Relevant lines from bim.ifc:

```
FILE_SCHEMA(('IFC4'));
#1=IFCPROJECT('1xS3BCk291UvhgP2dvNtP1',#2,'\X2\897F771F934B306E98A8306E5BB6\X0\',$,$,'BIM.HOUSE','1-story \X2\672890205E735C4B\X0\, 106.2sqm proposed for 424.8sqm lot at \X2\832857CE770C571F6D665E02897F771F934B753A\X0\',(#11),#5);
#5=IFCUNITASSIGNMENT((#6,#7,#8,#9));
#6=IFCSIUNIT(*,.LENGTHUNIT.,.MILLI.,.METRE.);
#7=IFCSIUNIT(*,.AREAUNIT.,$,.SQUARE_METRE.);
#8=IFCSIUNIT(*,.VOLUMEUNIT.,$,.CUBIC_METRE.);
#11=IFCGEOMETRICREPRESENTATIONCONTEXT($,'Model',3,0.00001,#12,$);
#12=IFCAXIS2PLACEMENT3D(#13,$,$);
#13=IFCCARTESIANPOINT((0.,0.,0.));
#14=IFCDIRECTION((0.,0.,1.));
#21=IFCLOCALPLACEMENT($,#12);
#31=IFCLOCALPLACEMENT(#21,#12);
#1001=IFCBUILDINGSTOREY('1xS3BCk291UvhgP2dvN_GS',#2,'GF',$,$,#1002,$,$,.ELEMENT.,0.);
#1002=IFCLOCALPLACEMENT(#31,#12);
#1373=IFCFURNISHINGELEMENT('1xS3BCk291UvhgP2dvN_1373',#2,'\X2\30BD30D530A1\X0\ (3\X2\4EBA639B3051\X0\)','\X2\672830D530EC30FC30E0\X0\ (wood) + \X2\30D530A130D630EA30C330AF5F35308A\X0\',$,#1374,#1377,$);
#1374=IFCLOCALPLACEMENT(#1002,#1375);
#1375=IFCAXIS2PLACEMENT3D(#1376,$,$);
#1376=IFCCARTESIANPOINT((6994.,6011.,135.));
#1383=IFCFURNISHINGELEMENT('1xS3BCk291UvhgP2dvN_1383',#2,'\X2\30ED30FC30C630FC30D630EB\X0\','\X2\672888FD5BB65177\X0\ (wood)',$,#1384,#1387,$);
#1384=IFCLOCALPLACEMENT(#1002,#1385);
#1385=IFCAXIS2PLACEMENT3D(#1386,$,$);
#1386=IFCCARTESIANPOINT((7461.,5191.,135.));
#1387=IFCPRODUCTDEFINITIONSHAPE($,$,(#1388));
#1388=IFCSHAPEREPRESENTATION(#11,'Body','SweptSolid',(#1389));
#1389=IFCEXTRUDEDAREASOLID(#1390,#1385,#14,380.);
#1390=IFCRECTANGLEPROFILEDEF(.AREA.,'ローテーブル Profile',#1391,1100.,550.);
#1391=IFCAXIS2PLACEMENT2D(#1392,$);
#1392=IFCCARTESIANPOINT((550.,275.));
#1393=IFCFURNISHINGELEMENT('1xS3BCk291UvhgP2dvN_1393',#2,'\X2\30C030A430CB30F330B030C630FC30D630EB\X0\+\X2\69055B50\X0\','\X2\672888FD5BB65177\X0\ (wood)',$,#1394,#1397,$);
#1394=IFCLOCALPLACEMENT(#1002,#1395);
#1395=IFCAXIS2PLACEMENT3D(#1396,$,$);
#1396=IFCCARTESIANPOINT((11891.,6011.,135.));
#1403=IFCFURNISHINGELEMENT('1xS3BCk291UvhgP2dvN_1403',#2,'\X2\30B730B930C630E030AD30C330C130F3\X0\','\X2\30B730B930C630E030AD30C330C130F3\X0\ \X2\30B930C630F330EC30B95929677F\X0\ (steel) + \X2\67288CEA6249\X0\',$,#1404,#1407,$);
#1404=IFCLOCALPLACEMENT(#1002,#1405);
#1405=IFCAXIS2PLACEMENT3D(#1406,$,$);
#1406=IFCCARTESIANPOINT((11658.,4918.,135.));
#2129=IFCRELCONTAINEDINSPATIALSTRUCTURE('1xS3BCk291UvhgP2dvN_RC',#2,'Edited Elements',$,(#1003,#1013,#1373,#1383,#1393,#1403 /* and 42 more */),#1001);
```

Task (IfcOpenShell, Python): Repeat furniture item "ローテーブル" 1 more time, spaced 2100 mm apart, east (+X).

```python
import numpy as np
import ifcopenshell
import ifcopenshell.api.geometry
import ifcopenshell.api.root
import ifcopenshell.util.element
import ifcopenshell.util.placement

model = ifcopenshell.open("bim.ifc")


def reuse_history(source, copy):
    """copy_class also copies each property set's owner history, people and application; keep the originals."""
    for rel in copy.IsDefinedBy:
        if rel.is_a("IfcRelDefinesByProperties") and (history := rel.RelatingPropertyDefinition.OwnerHistory):
            rel.RelatingPropertyDefinition.OwnerHistory = source.OwnerHistory
            ifcopenshell.util.element.remove_deep2(model, history)


source = model.by_guid("1xS3BCk291UvhgP2dvN_1383")
base = ifcopenshell.util.placement.get_local_placement(source.ObjectPlacement)
step = np.array([1.0, 0.0, 0.0]) * 2100.0

for i in range(1, 2):
    copy = ifcopenshell.api.root.copy_class(model, product=source)
    copy.Representation = ifcopenshell.util.element.copy_deep(
        model, source.Representation, exclude=["IfcGeometricRepresentationContext", "IfcRepresentationMap"]
    )
    reuse_history(source, copy)
    matrix = base.copy()
    matrix[:3, 3] += i * step
    print("added at", matrix[:3, 3].round(3) + 0.0)
    ifcopenshell.api.geometry.edit_object_placement(model, product=copy, matrix=matrix, is_si=False)

model.write("bim_updated.ifc")
```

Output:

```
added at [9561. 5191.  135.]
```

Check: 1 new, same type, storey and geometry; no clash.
